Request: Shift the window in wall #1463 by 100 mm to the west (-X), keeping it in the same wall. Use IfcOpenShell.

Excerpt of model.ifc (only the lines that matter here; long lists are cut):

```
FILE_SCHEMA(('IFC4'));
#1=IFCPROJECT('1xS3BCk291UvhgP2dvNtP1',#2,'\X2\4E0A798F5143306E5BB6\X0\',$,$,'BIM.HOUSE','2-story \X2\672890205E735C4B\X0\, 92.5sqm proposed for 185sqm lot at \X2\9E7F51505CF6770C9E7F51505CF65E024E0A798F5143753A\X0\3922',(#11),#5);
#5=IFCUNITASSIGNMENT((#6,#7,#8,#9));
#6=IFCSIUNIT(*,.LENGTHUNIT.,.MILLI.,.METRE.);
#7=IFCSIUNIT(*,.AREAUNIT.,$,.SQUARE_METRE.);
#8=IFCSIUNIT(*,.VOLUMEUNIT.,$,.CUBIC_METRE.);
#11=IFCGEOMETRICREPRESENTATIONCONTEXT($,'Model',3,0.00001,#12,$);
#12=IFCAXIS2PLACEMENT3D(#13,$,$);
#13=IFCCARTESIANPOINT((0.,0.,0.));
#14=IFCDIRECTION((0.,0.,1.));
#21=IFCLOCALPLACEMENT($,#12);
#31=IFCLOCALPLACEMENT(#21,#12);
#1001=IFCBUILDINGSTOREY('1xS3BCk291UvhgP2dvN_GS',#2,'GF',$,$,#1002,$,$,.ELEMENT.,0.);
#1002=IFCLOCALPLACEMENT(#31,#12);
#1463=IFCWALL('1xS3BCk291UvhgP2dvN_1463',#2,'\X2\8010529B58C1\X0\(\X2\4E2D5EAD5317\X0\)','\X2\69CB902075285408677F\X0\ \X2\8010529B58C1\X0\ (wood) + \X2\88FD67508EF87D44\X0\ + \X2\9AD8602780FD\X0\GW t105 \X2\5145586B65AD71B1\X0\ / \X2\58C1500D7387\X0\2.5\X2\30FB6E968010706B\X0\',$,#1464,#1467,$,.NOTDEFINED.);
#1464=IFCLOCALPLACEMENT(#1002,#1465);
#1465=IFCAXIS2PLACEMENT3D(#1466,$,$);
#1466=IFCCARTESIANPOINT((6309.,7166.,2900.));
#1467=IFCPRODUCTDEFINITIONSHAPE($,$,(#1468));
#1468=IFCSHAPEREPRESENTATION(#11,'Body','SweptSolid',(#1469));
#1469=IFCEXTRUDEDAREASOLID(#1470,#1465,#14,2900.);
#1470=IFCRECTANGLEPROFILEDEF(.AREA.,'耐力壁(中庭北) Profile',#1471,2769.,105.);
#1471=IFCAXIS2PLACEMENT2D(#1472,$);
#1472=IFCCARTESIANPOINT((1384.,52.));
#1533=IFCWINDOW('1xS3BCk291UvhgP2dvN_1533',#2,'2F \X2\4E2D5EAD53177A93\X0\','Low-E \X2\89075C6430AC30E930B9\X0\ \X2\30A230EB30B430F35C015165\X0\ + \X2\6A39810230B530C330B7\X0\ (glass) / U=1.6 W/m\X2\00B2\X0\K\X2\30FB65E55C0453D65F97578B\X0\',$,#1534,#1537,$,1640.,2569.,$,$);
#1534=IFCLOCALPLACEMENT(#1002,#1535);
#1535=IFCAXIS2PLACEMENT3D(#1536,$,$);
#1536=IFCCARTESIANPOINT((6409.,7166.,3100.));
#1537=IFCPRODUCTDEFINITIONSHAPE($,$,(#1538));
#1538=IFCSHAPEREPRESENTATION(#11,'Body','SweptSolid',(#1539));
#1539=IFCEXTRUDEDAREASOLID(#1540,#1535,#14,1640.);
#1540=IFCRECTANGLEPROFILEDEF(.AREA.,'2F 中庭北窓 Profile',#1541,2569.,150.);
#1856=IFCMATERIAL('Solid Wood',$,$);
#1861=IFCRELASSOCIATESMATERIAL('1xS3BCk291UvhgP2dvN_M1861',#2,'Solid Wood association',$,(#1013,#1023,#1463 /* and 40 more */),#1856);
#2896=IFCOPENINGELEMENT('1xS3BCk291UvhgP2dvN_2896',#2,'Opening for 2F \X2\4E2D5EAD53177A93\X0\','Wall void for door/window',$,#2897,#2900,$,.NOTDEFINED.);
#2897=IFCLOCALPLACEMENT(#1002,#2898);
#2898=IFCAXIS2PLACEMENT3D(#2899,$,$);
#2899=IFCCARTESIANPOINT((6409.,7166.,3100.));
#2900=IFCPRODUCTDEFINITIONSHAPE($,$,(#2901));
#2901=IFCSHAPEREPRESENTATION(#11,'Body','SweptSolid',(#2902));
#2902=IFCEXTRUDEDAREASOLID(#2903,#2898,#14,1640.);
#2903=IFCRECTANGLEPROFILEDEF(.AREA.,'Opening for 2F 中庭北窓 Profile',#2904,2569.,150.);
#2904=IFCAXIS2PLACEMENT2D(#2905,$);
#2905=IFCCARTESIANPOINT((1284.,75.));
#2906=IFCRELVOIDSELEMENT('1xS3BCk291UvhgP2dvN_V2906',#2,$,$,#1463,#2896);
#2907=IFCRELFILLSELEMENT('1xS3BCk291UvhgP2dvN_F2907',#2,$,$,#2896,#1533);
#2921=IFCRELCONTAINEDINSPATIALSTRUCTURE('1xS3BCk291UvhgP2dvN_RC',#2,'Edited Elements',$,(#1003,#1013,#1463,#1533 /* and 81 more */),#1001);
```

```python
import ifcopenshell
import ifcopenshell.api.geometry
import ifcopenshell.util.placement
import ifcopenshell.util.unit

model = ifcopenshell.open("model.ifc")
unit_scale = ifcopenshell.util.unit.calculate_unit_scale(model)

window = model.by_id(1533)
opening = window.FillsVoids[0].RelatingOpeningElement
wall = opening.VoidsElements[0].RelatingBuildingElement

wall_matrix = ifcopenshell.util.placement.get_local_placement(wall.ObjectPlacement)
shift = wall_matrix[:3, 0] * -0.1 / unit_scale
before = ifcopenshell.util.placement.get_local_placement(window.ObjectPlacement)[:3, 3].copy()

# The window is not placed relative to its opening, so move both.
for product in (opening, window):
    matrix = ifcopenshell.util.placement.get_local_placement(product.ObjectPlacement)
    matrix[:3, 3] += shift
    ifcopenshell.api.geometry.edit_object_placement(model, product=product, matrix=matrix, is_si=False)

after = ifcopenshell.util.placement.get_local_placement(window.ObjectPlacement)[:3, 3]
print("window moved by", (after - before).round(3) + 0.0)

model.write("model-out.ifc")
```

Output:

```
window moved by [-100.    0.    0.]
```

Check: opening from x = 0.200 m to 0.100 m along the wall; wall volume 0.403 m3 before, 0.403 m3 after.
